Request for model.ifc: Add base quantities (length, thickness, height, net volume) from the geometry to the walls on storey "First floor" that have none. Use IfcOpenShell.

First a look at what the model holds.

```python
import ifcopenshell
import ifcopenshell.util.element
import ifcopenshell.util.unit

model = ifcopenshell.open("model.ifc")
print(model.schema)
for unit_type in ("LENGTHUNIT", "AREAUNIT", "VOLUMEUNIT"):
    print(unit_type, ifcopenshell.util.unit.calculate_unit_scale(model, unit_type))
storey = next(s for s in model.by_type("IfcBuildingStorey") if s.Name == "First floor")
walls = [e for e in ifcopenshell.util.element.get_decomposition(storey) if e.is_a("IfcWall")]
for e in sorted(walls, key=lambda e: e.id()):
    print(e.id(), e.is_a(), e.Name, list(ifcopenshell.util.element.get_psets(e, qtos_only=True)), sep=" | ")
```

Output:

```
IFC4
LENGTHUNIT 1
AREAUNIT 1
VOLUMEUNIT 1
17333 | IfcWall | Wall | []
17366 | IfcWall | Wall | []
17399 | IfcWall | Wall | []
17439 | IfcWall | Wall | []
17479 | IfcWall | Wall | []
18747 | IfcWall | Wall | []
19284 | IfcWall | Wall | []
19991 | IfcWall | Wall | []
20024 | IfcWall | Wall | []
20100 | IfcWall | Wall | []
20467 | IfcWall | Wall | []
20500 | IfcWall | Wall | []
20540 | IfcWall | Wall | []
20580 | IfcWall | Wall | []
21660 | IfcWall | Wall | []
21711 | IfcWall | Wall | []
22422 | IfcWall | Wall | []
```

```python
import ifcopenshell
import ifcopenshell.api.pset
import ifcopenshell.geom
import ifcopenshell.util.element
import ifcopenshell.util.shape
import ifcopenshell.util.unit

model = ifcopenshell.open("model.ifc")
unit_scale = ifcopenshell.util.unit.calculate_unit_scale(model)
volume_scale = ifcopenshell.util.unit.calculate_unit_scale(model, "VOLUMEUNIT")
settings = ifcopenshell.geom.settings()

storey = next(s for s in model.by_type("IfcBuildingStorey") if s.Name == "First floor")
walls = [e for e in ifcopenshell.util.element.get_decomposition(storey) if e.is_a("IfcWall")]

for e in sorted(walls, key=lambda e: e.id()):
    if ifcopenshell.util.element.get_psets(e, qtos_only=True, should_inherit=False):
        continue
    # Geometry comes back in metres, in the element's own axes.
    shape = ifcopenshell.geom.create_shape(settings, e)
    values = {
        "Length": ifcopenshell.util.shape.get_x(shape.geometry) / unit_scale,
        "Width": ifcopenshell.util.shape.get_y(shape.geometry) / unit_scale,
        "Height": ifcopenshell.util.shape.get_z(shape.geometry) / unit_scale,
        "NetVolume": ifcopenshell.util.shape.get_volume(shape.geometry) / volume_scale,
    }
    qto = ifcopenshell.api.pset.add_qto(model, product=e, name="Qto_WallBaseQuantities")
    ifcopenshell.api.pset.edit_qto(model, qto=qto, properties=values)
    print(e.id(), {k: round(v, 3) for k, v in values.items()})

model.write("model_rev.ifc")
```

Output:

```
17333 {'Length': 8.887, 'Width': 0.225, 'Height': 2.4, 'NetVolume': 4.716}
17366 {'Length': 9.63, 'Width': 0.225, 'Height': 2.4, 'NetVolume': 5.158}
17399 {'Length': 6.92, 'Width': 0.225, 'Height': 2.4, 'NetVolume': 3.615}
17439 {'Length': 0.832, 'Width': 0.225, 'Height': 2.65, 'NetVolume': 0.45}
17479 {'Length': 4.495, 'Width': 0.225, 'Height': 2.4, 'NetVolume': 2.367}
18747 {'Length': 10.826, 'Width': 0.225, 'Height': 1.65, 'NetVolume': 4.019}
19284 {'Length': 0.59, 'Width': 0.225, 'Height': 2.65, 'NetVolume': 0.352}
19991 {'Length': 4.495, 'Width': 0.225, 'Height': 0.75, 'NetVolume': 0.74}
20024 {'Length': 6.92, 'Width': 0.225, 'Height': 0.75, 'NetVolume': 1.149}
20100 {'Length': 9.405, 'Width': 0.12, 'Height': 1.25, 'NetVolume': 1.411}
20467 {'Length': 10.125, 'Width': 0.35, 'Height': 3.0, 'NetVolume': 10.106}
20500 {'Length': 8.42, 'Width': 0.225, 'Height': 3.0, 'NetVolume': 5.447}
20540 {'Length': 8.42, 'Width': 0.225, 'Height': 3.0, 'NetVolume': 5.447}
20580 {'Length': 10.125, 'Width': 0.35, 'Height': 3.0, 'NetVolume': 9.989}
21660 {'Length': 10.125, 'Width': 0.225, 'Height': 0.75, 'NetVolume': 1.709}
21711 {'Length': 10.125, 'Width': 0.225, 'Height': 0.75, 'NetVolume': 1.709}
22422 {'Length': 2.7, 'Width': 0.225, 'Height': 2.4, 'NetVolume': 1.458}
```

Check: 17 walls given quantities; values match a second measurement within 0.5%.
